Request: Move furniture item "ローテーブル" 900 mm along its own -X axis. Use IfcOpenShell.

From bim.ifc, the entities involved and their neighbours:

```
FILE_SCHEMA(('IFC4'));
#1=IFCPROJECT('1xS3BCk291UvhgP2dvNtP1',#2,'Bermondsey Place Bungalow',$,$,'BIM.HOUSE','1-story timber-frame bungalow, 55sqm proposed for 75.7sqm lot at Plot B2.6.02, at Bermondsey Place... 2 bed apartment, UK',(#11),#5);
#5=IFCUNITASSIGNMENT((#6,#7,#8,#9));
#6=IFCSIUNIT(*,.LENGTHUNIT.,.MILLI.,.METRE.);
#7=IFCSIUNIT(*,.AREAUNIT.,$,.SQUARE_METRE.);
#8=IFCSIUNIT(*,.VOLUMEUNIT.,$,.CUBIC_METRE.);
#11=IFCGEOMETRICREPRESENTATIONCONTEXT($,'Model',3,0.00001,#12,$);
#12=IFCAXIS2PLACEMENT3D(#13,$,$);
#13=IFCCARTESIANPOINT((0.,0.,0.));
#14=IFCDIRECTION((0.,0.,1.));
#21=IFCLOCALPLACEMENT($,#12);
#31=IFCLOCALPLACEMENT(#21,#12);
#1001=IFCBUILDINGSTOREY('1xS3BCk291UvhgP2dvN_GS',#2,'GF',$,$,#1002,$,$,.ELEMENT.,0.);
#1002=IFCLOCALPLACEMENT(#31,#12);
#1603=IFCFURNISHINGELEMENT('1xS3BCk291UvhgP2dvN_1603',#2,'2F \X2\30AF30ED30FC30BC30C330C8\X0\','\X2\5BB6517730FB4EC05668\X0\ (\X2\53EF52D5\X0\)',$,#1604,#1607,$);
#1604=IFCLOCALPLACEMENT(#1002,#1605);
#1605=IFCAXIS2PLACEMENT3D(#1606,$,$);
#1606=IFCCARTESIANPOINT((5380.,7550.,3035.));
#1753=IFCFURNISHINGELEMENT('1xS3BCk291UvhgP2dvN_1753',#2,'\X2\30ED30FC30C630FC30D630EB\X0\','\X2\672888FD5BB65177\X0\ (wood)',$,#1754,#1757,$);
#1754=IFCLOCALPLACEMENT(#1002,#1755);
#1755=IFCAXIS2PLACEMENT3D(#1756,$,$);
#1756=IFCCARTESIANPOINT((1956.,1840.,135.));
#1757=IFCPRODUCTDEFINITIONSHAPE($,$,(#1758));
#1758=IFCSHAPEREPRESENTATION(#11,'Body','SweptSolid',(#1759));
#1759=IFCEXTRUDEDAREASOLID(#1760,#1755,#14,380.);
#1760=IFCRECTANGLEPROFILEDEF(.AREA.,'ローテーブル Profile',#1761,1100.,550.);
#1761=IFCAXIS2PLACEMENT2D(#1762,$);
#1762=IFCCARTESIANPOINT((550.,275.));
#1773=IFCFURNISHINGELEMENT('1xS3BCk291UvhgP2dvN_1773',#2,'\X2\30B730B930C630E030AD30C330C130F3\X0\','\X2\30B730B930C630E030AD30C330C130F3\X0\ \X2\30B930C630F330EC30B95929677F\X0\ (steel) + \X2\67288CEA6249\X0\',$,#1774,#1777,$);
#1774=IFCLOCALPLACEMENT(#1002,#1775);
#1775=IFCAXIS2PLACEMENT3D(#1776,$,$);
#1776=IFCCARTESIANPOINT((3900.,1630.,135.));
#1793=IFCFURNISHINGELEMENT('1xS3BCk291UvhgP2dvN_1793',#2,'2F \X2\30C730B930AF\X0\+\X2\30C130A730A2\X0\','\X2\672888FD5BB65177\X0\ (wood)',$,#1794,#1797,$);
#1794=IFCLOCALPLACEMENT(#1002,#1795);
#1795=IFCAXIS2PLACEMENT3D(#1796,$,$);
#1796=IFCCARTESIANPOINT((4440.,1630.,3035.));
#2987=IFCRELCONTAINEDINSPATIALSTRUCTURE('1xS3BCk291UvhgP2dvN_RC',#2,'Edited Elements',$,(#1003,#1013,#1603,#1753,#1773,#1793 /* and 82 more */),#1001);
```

```python
import ifcopenshell
import ifcopenshell.api.geometry
import ifcopenshell.util.placement

model = ifcopenshell.open("bim.ifc")

item = model.by_guid("1xS3BCk291UvhgP2dvN_1753")
matrix = ifcopenshell.util.placement.get_local_placement(item.ObjectPlacement)
matrix[:3, 3] -= matrix[:3, 0] * 900.0
ifcopenshell.api.geometry.edit_object_placement(model, product=item, matrix=matrix, is_si=False)

print(ifcopenshell.util.placement.get_local_placement(item.ObjectPlacement).round(3) + 0.0)

model.write("bim_edited.ifc")
```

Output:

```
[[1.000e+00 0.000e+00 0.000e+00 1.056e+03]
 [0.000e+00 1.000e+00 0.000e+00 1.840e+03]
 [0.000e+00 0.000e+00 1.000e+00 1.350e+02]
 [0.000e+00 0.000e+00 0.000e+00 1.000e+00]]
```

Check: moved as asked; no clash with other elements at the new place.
